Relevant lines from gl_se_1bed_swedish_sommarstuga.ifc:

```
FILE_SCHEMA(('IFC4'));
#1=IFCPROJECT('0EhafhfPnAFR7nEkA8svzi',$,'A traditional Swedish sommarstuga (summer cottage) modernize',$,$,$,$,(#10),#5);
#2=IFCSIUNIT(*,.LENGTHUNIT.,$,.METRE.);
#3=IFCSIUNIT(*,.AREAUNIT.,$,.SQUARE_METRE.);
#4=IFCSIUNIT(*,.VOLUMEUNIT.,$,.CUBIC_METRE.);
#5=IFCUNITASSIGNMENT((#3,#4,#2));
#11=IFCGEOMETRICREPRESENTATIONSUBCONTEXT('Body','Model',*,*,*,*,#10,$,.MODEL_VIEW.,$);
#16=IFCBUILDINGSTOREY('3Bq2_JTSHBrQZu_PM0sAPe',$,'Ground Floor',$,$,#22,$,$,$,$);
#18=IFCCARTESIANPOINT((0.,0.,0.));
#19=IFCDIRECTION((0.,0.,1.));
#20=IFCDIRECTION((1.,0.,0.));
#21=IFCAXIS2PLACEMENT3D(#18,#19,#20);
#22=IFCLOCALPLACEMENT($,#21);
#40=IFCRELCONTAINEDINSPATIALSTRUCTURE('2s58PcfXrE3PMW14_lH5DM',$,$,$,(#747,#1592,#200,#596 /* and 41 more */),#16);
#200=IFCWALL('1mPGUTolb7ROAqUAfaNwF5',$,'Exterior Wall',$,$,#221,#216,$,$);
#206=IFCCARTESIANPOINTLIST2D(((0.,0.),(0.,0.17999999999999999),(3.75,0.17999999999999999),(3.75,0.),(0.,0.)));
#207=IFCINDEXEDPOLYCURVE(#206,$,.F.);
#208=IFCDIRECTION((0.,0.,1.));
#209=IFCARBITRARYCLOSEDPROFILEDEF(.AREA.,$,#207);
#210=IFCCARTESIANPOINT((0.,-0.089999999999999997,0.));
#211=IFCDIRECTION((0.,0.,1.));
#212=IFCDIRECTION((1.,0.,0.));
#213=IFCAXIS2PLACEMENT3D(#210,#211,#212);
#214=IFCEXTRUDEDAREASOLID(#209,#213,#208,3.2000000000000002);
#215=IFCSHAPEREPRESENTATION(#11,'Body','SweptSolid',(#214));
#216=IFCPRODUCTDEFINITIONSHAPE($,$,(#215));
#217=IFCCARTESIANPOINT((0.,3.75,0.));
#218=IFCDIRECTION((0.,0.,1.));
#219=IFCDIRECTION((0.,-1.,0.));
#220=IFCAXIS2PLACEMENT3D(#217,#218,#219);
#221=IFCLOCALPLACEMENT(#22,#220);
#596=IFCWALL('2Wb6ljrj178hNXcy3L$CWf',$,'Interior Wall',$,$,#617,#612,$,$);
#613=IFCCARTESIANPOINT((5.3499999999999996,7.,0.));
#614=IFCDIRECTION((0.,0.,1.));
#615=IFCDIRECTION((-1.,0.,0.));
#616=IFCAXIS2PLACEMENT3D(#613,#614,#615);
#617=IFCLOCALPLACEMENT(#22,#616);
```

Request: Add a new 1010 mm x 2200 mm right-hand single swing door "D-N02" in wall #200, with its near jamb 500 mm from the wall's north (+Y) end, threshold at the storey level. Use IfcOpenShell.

```python
import numpy as np
import ifcopenshell
import ifcopenshell.api.feature
import ifcopenshell.api.geometry
import ifcopenshell.api.root
import ifcopenshell.api.spatial
import ifcopenshell.geom
import ifcopenshell.util.element
import ifcopenshell.util.placement
import ifcopenshell.util.representation
import ifcopenshell.util.shape
import ifcopenshell.util.unit

model = ifcopenshell.open("gl_se_1bed_swedish_sommarstuga.ifc")
unit_scale = ifcopenshell.util.unit.calculate_unit_scale(model)
settings = ifcopenshell.geom.settings()


def volume(element):
    """Net volume in cubic metres, openings subtracted."""
    shape = ifcopenshell.geom.create_shape(settings, element)
    return ifcopenshell.util.shape.get_volume(shape.geometry)


wall = model.by_guid("1mPGUTolb7ROAqUAfaNwF5")
storey = ifcopenshell.util.element.get_container(wall, ifc_class="IfcBuildingStorey")
context = ifcopenshell.util.representation.get_context(model, "Model", "Body", "MODEL_VIEW")
before = volume(wall)

width, height, from_end, sill = 1.01, 2.2, 0.5, 0.0  # metres

# The wall runs along its own X axis, and the end named is its -X end.
wall_shape = ifcopenshell.geom.create_shape(settings, wall)
x, y, z = ifcopenshell.util.shape.get_vertices(wall_shape.geometry).T
start = x.min() + from_end
face, thickness = float(y.min()), float(y.max() - y.min())
wall_matrix = ifcopenshell.util.placement.get_local_placement(wall.ObjectPlacement)
level = ifcopenshell.util.placement.get_local_placement(storey.ObjectPlacement)[2, 3]


def in_wall(x, y):
    """Placement at x, y metres in the wall's axes, at sill height."""
    matrix = wall_matrix.copy()
    matrix[:, 3] = wall_matrix @ np.array([x / unit_scale, y / unit_scale, 0.0, 1.0])
    matrix[2, 3] = level + sill / unit_scale
    return matrix


# Opening: a box that overshoots both wall faces by 50 mm.
opening = ifcopenshell.api.root.create_entity(model, ifc_class="IfcOpeningElement", predefined_type="OPENING")
box = ifcopenshell.api.geometry.add_wall_representation(
    model, context=context, length=width, height=height, thickness=thickness + 0.1
)
ifcopenshell.api.geometry.assign_representation(model, product=opening, representation=box)
ifcopenshell.api.geometry.edit_object_placement(model, product=opening, matrix=in_wall(start, face - 0.05), is_si=False)
ifcopenshell.api.feature.add_feature(model, feature=opening, element=wall)

door = ifcopenshell.api.root.create_entity(model, ifc_class="IfcDoor", name="D-N02", predefined_type="DOOR")
door.OverallWidth, door.OverallHeight = width / unit_scale, height / unit_scale
door.OperationType = "SINGLE_SWING_RIGHT"
body = ifcopenshell.api.geometry.add_door_representation(
    model,
    context=context,
    overall_width=door.OverallWidth,
    overall_height=door.OverallHeight,
    operation_type="SINGLE_SWING_RIGHT",
    lining_properties={"LiningDepth": thickness / unit_scale, "ThresholdDepth": thickness / unit_scale},
)
ifcopenshell.api.geometry.assign_representation(model, product=door, representation=body)
ifcopenshell.api.spatial.assign_container(model, products=[door], relating_structure=storey)
ifcopenshell.api.feature.add_filling(model, opening=opening, element=door)

# The lining spans the wall, so the door starts at the wall face.
ifcopenshell.api.geometry.edit_object_placement(model, product=door, matrix=in_wall(start, face), is_si=False)

after = volume(wall)

print(f"wall volume {before:.3f} -> {after:.3f} m3")

model.write("gl_se_1bed_swedish_sommarstuga-out.ifc")
```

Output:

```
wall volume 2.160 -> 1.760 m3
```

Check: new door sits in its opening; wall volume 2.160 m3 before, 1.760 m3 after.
